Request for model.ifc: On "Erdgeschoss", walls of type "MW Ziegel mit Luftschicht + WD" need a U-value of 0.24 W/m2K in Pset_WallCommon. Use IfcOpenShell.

First a look at what the model holds.

```python
import ifcopenshell
import ifcopenshell.util.element

model = ifcopenshell.open("model.ifc")
print(model.schema)
storey = next(s for s in model.by_type("IfcBuildingStorey") if s.Name == "Erdgeschoss")
walls = [e for e in ifcopenshell.util.element.get_decomposition(storey) if e.is_a("IfcWall")]
seen = {}
for e in walls:
    element_type = ifcopenshell.util.element.get_type(e)
    key = (element_type.Name if element_type != e and element_type else None, ifcopenshell.util.element.get_pset(e, "Pset_WallCommon", "ThermalTransmittance"))
    seen[key] = seen.get(key, 0) + 1
for (name, value), count in sorted(seen.items(), key=str):
    print(count, "x", name, "|", value)
```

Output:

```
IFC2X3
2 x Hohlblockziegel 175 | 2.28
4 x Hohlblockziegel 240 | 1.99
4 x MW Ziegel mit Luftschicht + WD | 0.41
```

```python
import ifcopenshell
import ifcopenshell.api.pset
import ifcopenshell.util.element

model = ifcopenshell.open("model.ifc")

storey = next(s for s in model.by_type("IfcBuildingStorey") if s.Name == "Erdgeschoss")
walls = [e for e in ifcopenshell.util.element.get_decomposition(storey) if e.is_a("IfcWall")]

count = 0
for e in walls:
    element_type = ifcopenshell.util.element.get_type(e)
    if element_type in (None, e) or element_type.Name != "MW Ziegel mit Luftschicht + WD":
        continue
    # add_pset returns the element's existing set when there is one.
    pset = ifcopenshell.api.pset.add_pset(model, product=e, name="Pset_WallCommon")
    ifcopenshell.api.pset.edit_pset(model, pset=pset, properties={"ThermalTransmittance": 0.24})
    count += 1

print(count, "walls updated")

model.write("model_edited.ifc")
```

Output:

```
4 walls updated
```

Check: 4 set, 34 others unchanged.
